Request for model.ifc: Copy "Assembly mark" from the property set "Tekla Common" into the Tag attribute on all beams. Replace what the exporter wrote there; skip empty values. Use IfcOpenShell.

First a look at what the model holds.

```python
import ifcopenshell
import ifcopenshell.util.element

model = ifcopenshell.open("model.ifc")
print(model.schema)
beams = model.by_type("IfcBeam")
print(len(beams), "beams")
for e in beams[:8]:
    source = ifcopenshell.util.element.get_pset(e, "Tekla Common", "Assembly mark")
    target = e.Tag
    print(e.id(), repr(source), repr(target), sep=" | ")
```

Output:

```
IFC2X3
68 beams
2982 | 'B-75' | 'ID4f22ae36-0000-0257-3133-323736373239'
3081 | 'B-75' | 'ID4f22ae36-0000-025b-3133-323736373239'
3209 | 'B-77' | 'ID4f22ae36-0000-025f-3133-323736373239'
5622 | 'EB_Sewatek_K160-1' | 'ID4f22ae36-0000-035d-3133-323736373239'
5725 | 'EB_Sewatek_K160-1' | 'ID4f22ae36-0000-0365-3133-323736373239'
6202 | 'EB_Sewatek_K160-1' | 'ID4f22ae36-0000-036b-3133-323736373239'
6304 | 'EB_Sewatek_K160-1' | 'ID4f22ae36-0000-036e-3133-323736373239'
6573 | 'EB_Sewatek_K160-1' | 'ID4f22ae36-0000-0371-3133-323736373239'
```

```python
import ifcopenshell
import ifcopenshell.util.element

model = ifcopenshell.open("model.ifc")

count = 0
for e in model.by_type("IfcBeam"):
    value = ifcopenshell.util.element.get_pset(e, "Tekla Common", "Assembly mark")
    current = e.Tag
    if not value or not value.strip() or current == value:
        continue
    e.Tag = value
    count += 1

print(count, "beams updated")

model.write("model-out.ifc")
```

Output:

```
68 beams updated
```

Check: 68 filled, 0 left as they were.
